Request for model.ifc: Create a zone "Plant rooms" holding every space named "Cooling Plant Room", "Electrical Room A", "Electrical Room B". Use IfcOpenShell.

First a look at what the model holds.

```python
import ifcopenshell

model = ifcopenshell.open("model.ifc")
print(model.schema)
seen = {}
for space in model.by_type("IfcSpace"):
    seen[space.LongName] = seen.get(space.LongName, 0) + 1
for name, count in sorted(seen.items(), key=str):
    print(count, "x", name)
print("zones:", [z.Name for z in model.by_type("IfcZone")][:20])
```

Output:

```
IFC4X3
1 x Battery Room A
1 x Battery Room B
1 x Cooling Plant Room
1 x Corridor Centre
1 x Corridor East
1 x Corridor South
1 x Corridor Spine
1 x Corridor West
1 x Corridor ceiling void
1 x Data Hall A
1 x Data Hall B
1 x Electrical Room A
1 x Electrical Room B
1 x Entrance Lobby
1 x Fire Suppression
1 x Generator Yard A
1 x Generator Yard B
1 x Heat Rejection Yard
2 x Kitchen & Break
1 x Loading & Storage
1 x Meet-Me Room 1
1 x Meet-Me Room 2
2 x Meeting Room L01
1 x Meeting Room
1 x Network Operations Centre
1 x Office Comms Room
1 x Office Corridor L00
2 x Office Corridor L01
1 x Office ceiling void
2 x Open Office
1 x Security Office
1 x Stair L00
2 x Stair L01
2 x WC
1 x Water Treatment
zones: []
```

```python
import ifcopenshell
import ifcopenshell.api.group
import ifcopenshell.api.root

model = ifcopenshell.open("model.ifc")

names = {"Cooling Plant Room", "Electrical Room A", "Electrical Room B"}
spaces = [s for s in model.by_type("IfcSpace") if s.LongName in names]

zone = ifcopenshell.api.root.create_entity(model, ifc_class="IfcZone", name="Plant rooms")
ifcopenshell.api.group.assign_group(model, products=spaces, group=zone)
print(len(spaces), "spaces in", zone.Name)

model.write("model_updated.ifc")
```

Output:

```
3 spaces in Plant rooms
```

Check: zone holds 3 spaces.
